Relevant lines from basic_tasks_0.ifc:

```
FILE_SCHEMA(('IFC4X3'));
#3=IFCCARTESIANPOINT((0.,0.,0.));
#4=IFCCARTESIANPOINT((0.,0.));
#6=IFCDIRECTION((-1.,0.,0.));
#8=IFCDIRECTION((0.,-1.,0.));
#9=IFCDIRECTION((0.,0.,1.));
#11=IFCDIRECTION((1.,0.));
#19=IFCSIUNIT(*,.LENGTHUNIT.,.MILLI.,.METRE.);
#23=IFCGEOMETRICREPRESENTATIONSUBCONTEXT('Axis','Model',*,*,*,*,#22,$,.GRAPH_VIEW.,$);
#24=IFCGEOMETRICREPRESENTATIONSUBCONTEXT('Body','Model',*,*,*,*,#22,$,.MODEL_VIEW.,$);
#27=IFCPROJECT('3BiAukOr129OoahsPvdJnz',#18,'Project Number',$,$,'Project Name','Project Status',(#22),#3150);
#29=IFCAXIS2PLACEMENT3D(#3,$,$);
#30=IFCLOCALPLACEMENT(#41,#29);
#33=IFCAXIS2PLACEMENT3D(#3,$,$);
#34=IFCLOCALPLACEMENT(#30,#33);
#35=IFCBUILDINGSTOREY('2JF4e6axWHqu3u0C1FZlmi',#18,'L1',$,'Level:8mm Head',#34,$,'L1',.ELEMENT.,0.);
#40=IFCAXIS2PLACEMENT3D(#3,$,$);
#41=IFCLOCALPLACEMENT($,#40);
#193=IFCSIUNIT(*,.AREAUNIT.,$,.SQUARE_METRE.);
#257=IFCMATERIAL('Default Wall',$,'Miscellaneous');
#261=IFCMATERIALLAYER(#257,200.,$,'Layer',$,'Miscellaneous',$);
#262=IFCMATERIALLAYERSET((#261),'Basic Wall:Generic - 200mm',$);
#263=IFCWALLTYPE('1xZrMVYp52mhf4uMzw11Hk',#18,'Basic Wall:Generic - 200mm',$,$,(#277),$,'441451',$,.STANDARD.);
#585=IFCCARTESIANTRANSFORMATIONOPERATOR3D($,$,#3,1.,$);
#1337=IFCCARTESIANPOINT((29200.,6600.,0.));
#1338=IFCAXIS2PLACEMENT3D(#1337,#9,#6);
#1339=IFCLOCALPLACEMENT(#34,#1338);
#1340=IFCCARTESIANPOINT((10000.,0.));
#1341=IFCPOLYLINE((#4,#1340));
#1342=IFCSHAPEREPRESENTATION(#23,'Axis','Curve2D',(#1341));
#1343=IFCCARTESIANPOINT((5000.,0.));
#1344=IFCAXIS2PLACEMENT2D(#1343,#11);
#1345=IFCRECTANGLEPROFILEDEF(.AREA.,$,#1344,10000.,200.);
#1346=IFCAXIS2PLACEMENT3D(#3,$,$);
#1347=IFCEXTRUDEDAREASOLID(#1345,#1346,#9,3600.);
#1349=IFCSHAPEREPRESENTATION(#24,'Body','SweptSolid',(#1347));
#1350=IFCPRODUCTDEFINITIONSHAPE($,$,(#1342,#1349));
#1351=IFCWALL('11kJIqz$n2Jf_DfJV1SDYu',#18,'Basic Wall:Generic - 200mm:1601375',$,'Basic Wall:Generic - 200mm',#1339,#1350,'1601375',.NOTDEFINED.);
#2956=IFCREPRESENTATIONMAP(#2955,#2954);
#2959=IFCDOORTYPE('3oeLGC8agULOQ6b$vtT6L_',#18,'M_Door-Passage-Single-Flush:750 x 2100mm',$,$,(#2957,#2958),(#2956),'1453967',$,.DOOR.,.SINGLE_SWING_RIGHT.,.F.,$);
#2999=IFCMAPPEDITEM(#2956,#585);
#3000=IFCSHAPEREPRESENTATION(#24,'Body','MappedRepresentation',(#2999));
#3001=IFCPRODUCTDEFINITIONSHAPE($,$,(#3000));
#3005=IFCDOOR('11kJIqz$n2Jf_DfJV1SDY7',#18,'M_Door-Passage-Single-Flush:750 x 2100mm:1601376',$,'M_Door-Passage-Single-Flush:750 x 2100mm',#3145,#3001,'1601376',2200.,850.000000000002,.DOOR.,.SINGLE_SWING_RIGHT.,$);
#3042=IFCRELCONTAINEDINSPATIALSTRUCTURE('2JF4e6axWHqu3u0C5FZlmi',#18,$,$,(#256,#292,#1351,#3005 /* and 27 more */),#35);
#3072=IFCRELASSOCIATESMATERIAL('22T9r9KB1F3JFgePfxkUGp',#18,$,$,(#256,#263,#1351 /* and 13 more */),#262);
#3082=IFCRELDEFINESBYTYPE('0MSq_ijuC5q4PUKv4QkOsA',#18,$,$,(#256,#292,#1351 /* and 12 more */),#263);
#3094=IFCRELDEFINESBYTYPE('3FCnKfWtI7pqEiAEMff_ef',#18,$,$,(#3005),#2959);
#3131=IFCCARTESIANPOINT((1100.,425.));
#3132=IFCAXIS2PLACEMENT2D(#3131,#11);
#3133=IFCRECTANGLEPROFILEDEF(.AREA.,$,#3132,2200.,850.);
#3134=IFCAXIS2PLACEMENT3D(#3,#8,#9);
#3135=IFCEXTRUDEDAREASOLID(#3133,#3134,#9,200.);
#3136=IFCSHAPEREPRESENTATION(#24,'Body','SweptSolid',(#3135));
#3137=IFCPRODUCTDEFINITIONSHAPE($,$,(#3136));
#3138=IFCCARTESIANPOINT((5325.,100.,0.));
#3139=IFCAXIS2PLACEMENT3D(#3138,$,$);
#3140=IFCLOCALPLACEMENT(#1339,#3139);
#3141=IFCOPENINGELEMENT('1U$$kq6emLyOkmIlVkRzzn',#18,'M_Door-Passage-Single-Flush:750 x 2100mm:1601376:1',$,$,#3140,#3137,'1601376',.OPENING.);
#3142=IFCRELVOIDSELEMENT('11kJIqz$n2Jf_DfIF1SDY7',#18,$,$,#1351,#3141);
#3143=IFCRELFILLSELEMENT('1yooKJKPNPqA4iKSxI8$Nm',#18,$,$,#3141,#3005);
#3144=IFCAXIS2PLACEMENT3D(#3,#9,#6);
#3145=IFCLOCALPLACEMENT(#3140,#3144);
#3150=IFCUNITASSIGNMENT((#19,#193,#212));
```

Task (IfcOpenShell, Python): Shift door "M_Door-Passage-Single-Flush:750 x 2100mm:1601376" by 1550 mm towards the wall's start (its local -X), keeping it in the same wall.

```python
import ifcopenshell
import ifcopenshell.api.geometry
import ifcopenshell.util.placement
import ifcopenshell.util.unit

model = ifcopenshell.open("basic_tasks_0.ifc")
unit_scale = ifcopenshell.util.unit.calculate_unit_scale(model)

door = model.by_guid("11kJIqz$n2Jf_DfJV1SDY7")
opening = door.FillsVoids[0].RelatingOpeningElement
wall = opening.VoidsElements[0].RelatingBuildingElement

wall_matrix = ifcopenshell.util.placement.get_local_placement(wall.ObjectPlacement)
shift = wall_matrix[:3, 0] * -1.55 / unit_scale
before = ifcopenshell.util.placement.get_local_placement(door.ObjectPlacement)[:3, 3].copy()

# The door is placed relative to its opening, so it follows when the opening moves.
matrix = ifcopenshell.util.placement.get_local_placement(opening.ObjectPlacement)
matrix[:3, 3] += shift
ifcopenshell.api.geometry.edit_object_placement(
    model, product=opening, matrix=matrix, is_si=False, should_transform_children=True
)

after = ifcopenshell.util.placement.get_local_placement(door.ObjectPlacement)[:3, 3]
print("door moved by", (after - before).round(3) + 0.0)

model.write("basic_tasks_0_updated.ifc")
```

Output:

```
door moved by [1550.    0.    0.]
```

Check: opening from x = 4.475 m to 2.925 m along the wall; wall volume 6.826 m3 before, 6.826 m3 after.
